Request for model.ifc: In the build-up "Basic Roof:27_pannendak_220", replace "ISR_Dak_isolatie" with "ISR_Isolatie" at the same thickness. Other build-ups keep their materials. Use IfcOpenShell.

First a look at what the model holds.

```python
import ifcopenshell
import ifcopenshell.util.element

model = ifcopenshell.open("model.ifc")
print(model.schema)
for layer_set in model.by_type("IfcMaterialLayerSet"):
    if layer_set.LayerSetName == "Basic Roof:27_pannendak_220":
        for layer in layer_set.MaterialLayers:
            print(layer.id(), layer.Material and layer.Material.Name, layer.LayerThickness, sep=" | ")
        print(len(ifcopenshell.util.element.get_elements_by_material(model, layer_set)), "elements and types use it")
print(sorted(m.Name for m in model.by_type("IfcMaterial") if m.Name)[:60])
```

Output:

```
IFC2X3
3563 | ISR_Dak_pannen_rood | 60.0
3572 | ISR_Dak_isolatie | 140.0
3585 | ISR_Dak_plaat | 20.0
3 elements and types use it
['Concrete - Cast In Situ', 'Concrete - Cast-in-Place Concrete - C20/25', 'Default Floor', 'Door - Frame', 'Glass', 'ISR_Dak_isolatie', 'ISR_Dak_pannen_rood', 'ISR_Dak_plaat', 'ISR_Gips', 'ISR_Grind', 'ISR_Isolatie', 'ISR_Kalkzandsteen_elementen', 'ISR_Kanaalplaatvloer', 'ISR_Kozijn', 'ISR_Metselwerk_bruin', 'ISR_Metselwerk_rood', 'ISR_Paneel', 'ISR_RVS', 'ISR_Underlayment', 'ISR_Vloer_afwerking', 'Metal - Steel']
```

```python
import ifcopenshell
import ifcopenshell.api.material

model = ifcopenshell.open("model.ifc")

layer_set = next(s for s in model.by_type("IfcMaterialLayerSet") if s.LayerSetName == "Basic Roof:27_pannendak_220")
layer = next(l for l in layer_set.MaterialLayers if l.Material and l.Material.Name == "ISR_Dak_isolatie")
material = next(m for m in model.by_type("IfcMaterial") if m.Name == "ISR_Isolatie")

# Point this one layer at the other material; renaming the old one would change it everywhere.
ifcopenshell.api.material.edit_layer(model, layer=layer, attributes={}, material=material)

print([l.Material.Name if l.Material else None for l in layer_set.MaterialLayers])

model.write("model_edited.ifc")
```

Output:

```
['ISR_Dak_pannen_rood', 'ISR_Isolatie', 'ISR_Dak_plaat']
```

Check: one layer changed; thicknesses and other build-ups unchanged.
